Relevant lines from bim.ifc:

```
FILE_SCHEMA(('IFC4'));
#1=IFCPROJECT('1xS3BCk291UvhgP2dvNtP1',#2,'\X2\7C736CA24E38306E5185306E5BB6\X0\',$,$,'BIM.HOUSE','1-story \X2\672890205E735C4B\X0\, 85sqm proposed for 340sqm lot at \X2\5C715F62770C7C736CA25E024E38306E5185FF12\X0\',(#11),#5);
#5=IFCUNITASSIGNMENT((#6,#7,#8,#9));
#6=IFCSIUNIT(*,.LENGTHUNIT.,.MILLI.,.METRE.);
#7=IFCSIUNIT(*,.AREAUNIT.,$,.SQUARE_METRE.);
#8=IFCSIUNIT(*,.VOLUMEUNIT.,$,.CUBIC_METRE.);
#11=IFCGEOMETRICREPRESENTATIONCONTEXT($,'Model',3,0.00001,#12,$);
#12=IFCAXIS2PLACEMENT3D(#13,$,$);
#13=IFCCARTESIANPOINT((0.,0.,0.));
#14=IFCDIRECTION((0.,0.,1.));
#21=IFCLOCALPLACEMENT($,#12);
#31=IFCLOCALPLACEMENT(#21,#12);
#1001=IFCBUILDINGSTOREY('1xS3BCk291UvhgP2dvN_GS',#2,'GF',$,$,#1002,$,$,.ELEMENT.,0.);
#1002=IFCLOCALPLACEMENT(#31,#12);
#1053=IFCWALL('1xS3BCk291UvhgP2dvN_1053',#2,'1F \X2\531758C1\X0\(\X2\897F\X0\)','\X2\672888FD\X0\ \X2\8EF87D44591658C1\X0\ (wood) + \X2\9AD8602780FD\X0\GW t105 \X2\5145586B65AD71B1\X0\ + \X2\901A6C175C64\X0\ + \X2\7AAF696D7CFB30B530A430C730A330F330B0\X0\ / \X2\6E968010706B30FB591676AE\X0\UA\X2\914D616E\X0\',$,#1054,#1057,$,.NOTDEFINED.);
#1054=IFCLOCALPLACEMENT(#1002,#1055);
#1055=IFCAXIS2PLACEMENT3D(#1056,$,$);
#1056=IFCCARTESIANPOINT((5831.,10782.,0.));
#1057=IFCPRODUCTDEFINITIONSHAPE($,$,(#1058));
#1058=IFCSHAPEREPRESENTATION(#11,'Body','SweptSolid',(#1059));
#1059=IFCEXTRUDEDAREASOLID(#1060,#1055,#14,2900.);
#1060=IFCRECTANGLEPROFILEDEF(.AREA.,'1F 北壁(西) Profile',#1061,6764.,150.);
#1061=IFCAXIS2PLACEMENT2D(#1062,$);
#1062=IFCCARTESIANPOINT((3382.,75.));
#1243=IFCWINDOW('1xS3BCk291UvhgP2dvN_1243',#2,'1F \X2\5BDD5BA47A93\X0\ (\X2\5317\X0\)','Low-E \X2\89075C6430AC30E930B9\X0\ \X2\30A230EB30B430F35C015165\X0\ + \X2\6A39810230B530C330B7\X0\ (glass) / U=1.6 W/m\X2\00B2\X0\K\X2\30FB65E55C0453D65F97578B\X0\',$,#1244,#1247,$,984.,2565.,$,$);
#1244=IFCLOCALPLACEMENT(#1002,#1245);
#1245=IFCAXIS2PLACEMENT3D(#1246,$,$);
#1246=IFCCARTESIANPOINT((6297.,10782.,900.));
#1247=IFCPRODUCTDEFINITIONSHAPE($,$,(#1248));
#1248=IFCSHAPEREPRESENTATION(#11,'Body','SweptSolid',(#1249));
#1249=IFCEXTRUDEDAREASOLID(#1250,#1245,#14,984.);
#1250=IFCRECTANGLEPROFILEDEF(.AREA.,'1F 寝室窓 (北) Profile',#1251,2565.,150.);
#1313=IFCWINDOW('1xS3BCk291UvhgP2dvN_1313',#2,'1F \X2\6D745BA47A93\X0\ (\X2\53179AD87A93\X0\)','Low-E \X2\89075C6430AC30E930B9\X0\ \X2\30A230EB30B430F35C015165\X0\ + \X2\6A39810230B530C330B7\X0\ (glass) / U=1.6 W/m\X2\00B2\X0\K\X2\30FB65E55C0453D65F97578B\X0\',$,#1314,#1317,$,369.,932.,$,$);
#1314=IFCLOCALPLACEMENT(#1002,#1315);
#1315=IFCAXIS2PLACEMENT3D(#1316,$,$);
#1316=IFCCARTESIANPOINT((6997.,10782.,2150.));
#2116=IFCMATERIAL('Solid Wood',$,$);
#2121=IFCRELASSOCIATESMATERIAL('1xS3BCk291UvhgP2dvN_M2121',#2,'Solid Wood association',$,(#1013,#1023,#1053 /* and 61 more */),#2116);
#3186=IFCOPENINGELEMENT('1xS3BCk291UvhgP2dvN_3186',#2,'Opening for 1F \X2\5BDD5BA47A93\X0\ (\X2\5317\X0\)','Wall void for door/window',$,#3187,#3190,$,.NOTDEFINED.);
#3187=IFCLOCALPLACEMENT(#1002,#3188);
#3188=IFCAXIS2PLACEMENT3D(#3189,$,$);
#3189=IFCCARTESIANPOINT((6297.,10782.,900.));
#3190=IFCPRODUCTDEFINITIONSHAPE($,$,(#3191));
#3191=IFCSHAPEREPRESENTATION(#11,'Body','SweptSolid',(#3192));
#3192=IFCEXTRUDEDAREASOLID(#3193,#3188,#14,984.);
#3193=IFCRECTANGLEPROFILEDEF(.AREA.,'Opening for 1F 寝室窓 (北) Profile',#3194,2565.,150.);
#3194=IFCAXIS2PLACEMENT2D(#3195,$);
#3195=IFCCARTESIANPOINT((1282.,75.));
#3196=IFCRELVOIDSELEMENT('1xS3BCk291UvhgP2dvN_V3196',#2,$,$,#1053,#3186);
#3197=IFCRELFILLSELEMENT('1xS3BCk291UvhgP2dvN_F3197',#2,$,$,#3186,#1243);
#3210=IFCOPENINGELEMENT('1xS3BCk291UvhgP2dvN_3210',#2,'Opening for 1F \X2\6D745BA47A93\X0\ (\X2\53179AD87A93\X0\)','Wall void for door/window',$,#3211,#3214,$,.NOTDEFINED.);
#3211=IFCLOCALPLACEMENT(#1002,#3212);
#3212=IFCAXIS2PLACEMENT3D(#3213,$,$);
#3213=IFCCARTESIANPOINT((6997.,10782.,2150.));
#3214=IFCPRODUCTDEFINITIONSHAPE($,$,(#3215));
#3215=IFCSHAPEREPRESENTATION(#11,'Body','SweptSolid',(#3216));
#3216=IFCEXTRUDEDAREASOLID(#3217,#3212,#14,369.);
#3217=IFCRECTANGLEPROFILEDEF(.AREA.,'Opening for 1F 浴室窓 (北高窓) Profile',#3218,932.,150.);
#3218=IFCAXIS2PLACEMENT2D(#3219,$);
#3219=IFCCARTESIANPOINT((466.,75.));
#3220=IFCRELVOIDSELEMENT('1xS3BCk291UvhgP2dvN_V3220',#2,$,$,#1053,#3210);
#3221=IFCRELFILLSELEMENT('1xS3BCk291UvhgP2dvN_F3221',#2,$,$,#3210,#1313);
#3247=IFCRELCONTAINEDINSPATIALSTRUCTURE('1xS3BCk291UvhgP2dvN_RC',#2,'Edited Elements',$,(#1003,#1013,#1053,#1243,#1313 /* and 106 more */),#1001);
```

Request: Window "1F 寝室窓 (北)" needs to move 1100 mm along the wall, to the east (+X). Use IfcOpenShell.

```python
import ifcopenshell
import ifcopenshell.api.geometry
import ifcopenshell.util.placement

model = ifcopenshell.open("bim.ifc")

window = model.by_id(1243)
opening = window.FillsVoids[0].RelatingOpeningElement
wall = opening.VoidsElements[0].RelatingBuildingElement

wall_matrix = ifcopenshell.util.placement.get_local_placement(wall.ObjectPlacement)
shift = wall_matrix[:3, 0] * 1100.0
before = ifcopenshell.util.placement.get_local_placement(window.ObjectPlacement)[:3, 3].copy()

# The window is not placed relative to its opening, so move both.
for product in (opening, window):
    matrix = ifcopenshell.util.placement.get_local_placement(product.ObjectPlacement)
    matrix[:3, 3] += shift
    ifcopenshell.api.geometry.edit_object_placement(model, product=product, matrix=matrix, is_si=False)

after = ifcopenshell.util.placement.get_local_placement(window.ObjectPlacement)[:3, 3]
print("window moved by", (after - before).round(3) + 0.0)

model.write("bim_edited.ifc")
```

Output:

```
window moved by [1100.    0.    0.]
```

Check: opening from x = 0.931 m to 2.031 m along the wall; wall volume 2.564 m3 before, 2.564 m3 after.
